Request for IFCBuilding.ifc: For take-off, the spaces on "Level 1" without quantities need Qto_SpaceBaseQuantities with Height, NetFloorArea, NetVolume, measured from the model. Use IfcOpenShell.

First a look at what the model holds.

```python
import ifcopenshell
import ifcopenshell.util.element
import ifcopenshell.util.unit

model = ifcopenshell.open("IFCBuilding.ifc")
print(model.schema)
for unit_type in ("LENGTHUNIT", "AREAUNIT", "VOLUMEUNIT"):
    print(unit_type, ifcopenshell.util.unit.calculate_unit_scale(model, unit_type))
storey = next(s for s in model.by_type("IfcBuildingStorey") if s.Name == "Level 1")
spaces = [e for e in ifcopenshell.util.element.get_decomposition(storey) if e.is_a("IfcSpace")]
for e in sorted(spaces, key=lambda e: e.id()):
    print(e.id(), e.is_a(), e.Name, list(ifcopenshell.util.element.get_psets(e, qtos_only=True)), sep=" | ")
```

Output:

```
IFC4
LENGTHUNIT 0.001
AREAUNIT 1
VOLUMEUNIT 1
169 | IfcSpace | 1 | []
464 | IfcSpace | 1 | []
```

```python
import ifcopenshell
import ifcopenshell.api.pset
import ifcopenshell.geom
import ifcopenshell.util.element
import ifcopenshell.util.shape
import ifcopenshell.util.unit

model = ifcopenshell.open("IFCBuilding.ifc")
unit_scale = ifcopenshell.util.unit.calculate_unit_scale(model)
area_scale = ifcopenshell.util.unit.calculate_unit_scale(model, "AREAUNIT")
volume_scale = ifcopenshell.util.unit.calculate_unit_scale(model, "VOLUMEUNIT")
settings = ifcopenshell.geom.settings()

storey = next(s for s in model.by_type("IfcBuildingStorey") if s.Name == "Level 1")
spaces = [e for e in ifcopenshell.util.element.get_decomposition(storey) if e.is_a("IfcSpace")]

for e in sorted(spaces, key=lambda e: e.id()):
    if ifcopenshell.util.element.get_psets(e, qtos_only=True, should_inherit=False):
        continue
    # Geometry comes back in metres, in the element's own axes.
    shape = ifcopenshell.geom.create_shape(settings, e)
    values = {
        "Height": ifcopenshell.util.shape.get_z(shape.geometry) / unit_scale,
        "NetFloorArea": ifcopenshell.util.shape.get_footprint_area(shape.geometry) / area_scale,
        "NetVolume": ifcopenshell.util.shape.get_volume(shape.geometry) / volume_scale,
    }
    qto = ifcopenshell.api.pset.add_qto(model, product=e, name="Qto_SpaceBaseQuantities")
    ifcopenshell.api.pset.edit_qto(model, qto=qto, properties=values)
    print(e.id(), {k: round(v, 3) for k, v in values.items()})

model.write("IFCBuilding_updated.ifc")
```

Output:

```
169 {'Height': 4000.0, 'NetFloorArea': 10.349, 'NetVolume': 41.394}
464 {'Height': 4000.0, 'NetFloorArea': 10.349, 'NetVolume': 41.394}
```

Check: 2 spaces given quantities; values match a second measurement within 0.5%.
